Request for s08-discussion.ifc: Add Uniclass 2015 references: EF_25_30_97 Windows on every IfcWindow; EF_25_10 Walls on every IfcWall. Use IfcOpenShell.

First a look at what the model holds.

```python
import ifcopenshell

model = ifcopenshell.open("s08-discussion.ifc")
print(model.schema)
print("classifications:", [c.Name for c in model.by_type("IfcClassification")])
for ifc_class in ("IfcDoor", "IfcRoof", "IfcStair", "IfcWall", "IfcWindow"):
    print(ifc_class, len(model.by_type(ifc_class)))
```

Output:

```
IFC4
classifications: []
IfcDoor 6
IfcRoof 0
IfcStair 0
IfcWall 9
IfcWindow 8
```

```python
import ifcopenshell
import ifcopenshell.api.classification

model = ifcopenshell.open("s08-discussion.ifc")

system = ifcopenshell.api.classification.add_classification(model, classification="Uniclass 2015")

codes = {
    "IfcWindow": ("EF_25_30_97", "Windows"),
    "IfcWall": ("EF_25_10", "Walls"),
}
for ifc_class, (code, name) in codes.items():
    products = model.by_type(ifc_class)
    ifcopenshell.api.classification.add_reference(
        model, products=products, classification=system, identification=code, name=name
    )
    print(code, len(products))

model.write("s08-discussion_rev.ifc")
```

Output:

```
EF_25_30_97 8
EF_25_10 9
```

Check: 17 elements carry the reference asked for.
